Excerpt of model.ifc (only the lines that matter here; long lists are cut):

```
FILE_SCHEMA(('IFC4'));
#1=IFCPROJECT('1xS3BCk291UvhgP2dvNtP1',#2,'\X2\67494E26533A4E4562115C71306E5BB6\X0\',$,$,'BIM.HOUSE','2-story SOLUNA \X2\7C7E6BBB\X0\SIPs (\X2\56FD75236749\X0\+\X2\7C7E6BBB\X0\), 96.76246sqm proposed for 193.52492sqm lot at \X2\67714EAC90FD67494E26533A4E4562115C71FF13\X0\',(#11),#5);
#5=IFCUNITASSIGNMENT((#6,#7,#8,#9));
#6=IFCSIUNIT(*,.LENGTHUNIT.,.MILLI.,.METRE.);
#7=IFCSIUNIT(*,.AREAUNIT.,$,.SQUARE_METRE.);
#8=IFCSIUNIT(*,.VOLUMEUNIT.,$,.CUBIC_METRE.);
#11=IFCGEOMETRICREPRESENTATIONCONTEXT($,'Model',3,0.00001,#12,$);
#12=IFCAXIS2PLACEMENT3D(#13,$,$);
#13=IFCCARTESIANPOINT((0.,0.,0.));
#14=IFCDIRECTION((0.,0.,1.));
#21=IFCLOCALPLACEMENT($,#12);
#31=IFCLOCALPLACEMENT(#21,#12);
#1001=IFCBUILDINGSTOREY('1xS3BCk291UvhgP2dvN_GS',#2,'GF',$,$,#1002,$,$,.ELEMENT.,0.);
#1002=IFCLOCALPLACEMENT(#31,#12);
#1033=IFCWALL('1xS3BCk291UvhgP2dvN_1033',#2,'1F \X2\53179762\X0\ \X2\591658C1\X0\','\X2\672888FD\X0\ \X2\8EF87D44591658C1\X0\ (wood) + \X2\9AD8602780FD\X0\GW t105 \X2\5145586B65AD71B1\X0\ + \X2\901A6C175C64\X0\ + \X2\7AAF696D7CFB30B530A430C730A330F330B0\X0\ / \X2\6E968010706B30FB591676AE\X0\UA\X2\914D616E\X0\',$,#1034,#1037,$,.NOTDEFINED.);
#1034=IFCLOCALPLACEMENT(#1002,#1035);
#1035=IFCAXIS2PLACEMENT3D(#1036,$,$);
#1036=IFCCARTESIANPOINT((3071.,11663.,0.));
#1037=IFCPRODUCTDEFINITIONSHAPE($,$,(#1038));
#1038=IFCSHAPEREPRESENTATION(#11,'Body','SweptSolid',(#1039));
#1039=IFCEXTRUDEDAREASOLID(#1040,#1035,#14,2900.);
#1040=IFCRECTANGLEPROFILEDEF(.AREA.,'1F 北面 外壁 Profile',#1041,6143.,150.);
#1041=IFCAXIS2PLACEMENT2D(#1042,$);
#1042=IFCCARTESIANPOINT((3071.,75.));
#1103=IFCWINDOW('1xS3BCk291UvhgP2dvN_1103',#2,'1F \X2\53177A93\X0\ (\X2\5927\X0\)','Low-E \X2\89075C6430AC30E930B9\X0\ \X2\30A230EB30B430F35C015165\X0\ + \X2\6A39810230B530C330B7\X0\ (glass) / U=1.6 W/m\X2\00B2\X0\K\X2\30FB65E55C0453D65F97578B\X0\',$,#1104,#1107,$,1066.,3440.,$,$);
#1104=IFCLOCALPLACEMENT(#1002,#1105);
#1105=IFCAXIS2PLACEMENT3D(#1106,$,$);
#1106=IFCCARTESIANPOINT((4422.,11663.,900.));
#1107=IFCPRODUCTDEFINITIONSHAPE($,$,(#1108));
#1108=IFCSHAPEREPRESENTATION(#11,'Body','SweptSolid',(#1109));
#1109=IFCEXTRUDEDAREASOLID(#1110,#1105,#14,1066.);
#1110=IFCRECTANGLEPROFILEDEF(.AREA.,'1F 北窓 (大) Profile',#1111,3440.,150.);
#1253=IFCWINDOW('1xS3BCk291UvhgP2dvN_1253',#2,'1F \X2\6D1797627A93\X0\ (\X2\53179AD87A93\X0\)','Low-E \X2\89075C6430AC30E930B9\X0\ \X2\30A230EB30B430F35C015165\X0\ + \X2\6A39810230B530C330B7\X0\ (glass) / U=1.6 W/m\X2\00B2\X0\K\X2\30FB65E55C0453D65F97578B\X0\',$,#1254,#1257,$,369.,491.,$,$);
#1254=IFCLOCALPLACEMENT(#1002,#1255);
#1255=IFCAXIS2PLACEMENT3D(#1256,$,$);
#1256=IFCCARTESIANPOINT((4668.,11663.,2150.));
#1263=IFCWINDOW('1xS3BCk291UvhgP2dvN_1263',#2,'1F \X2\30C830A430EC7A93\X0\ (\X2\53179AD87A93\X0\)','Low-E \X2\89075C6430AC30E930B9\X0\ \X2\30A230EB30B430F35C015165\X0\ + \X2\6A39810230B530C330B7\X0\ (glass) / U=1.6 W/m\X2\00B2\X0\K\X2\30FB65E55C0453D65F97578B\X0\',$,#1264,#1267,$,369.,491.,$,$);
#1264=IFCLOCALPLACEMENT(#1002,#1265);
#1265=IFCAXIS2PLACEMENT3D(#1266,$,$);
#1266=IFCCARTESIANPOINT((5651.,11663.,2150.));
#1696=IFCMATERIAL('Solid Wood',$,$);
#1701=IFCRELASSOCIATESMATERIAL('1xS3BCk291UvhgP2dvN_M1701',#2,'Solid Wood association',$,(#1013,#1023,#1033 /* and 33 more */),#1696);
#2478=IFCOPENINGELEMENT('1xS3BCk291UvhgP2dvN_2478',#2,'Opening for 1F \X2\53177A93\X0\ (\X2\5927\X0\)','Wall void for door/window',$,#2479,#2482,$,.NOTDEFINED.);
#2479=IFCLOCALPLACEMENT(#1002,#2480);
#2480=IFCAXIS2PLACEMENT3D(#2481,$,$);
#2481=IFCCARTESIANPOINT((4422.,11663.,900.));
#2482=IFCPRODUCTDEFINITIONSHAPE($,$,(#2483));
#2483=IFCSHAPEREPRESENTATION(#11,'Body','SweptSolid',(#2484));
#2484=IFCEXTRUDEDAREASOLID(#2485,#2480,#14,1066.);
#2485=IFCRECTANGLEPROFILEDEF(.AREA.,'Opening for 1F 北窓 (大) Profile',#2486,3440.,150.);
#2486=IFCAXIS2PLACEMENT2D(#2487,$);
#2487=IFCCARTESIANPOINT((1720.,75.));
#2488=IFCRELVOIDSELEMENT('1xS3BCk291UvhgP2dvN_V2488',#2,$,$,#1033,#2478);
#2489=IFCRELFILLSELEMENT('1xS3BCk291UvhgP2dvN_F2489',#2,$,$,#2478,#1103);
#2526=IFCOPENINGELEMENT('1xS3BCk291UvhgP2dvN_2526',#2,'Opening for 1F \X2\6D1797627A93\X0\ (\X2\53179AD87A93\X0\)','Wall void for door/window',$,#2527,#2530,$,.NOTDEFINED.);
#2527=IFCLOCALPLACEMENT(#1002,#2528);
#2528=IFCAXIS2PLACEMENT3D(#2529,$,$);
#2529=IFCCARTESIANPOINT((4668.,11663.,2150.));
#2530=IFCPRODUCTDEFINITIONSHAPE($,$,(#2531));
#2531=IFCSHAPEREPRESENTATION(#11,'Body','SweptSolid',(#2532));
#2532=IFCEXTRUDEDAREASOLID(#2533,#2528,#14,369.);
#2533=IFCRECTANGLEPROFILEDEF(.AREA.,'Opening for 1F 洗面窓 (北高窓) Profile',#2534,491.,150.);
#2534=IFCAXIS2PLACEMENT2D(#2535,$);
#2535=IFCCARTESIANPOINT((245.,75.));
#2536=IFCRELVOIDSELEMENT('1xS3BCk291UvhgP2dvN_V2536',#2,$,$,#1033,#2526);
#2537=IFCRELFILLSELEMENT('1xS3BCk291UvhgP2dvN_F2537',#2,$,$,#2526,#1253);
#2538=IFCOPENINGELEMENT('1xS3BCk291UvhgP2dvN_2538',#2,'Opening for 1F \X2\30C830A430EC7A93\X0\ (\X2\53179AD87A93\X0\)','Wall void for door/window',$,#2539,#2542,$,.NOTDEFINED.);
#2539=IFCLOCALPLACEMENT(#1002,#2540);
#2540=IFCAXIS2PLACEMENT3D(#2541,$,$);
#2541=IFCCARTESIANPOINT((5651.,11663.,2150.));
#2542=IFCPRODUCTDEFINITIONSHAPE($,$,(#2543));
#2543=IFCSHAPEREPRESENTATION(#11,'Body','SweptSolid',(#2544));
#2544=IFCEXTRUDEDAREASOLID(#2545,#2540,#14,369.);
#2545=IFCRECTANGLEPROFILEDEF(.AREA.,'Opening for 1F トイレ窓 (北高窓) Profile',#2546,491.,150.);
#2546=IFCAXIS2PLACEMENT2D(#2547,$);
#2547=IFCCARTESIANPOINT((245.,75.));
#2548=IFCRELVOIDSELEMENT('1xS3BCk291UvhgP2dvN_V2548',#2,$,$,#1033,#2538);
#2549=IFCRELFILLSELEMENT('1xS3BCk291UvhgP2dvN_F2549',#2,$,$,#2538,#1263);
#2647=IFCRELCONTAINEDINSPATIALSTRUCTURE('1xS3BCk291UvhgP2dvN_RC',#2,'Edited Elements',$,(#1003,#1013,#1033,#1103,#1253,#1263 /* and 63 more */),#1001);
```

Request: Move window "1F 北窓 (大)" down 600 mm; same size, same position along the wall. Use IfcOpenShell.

```python
import numpy as np
import ifcopenshell
import ifcopenshell.api.geometry
import ifcopenshell.util.placement
import ifcopenshell.util.unit

model = ifcopenshell.open("model.ifc")
unit_scale = ifcopenshell.util.unit.calculate_unit_scale(model)

window = model.by_guid("1xS3BCk291UvhgP2dvN_1103")
opening = window.FillsVoids[0].RelatingOpeningElement
dz = -600.0

shift = np.array([0.0, 0.0, dz])
# The window is not placed relative to its opening, so move both.
for product in (opening, window):
    matrix = ifcopenshell.util.placement.get_local_placement(product.ObjectPlacement)
    matrix[:3, 3] += shift
    ifcopenshell.api.geometry.edit_object_placement(model, product=product, matrix=matrix, is_si=False)

print(f"moved by {dz * unit_scale:+.3f} m")

model.write("model-out.ifc")
```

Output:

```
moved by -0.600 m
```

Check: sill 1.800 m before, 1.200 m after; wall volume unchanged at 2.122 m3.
